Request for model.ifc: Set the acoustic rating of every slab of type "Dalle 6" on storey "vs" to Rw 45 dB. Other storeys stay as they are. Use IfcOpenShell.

First a look at what the model holds.

```python
import ifcopenshell
import ifcopenshell.util.element

model = ifcopenshell.open("model.ifc")
print(model.schema)
storey = next(s for s in model.by_type("IfcBuildingStorey") if s.Name == "vs")
slabs = [e for e in ifcopenshell.util.element.get_decomposition(storey) if e.is_a("IfcSlab")]
seen = {}
for e in slabs:
    element_type = ifcopenshell.util.element.get_type(e)
    key = (element_type.Name if element_type != e and element_type else None, ifcopenshell.util.element.get_pset(e, "Pset_SlabCommon", "AcousticRating"))
    seen[key] = seen.get(key, 0) + 1
for (name, value), count in sorted(seen.items(), key=str):
    print(count, "x", name, "|", value)
```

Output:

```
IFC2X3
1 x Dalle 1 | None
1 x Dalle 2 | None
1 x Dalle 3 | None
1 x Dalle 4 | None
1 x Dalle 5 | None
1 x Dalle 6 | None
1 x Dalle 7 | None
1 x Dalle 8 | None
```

```python
import ifcopenshell
import ifcopenshell.api.pset
import ifcopenshell.util.element

model = ifcopenshell.open("model.ifc")

storey = next(s for s in model.by_type("IfcBuildingStorey") if s.Name == "vs")
slabs = [e for e in ifcopenshell.util.element.get_decomposition(storey) if e.is_a("IfcSlab")]

count = 0
for e in slabs:
    element_type = ifcopenshell.util.element.get_type(e)
    if element_type in (None, e) or element_type.Name != "Dalle 6":
        continue
    # add_pset returns the element's existing set when there is one.
    pset = ifcopenshell.api.pset.add_pset(model, product=e, name="Pset_SlabCommon")
    ifcopenshell.api.pset.edit_pset(model, pset=pset, properties={"AcousticRating": "Rw 45 dB"})
    count += 1

print(count, "slabs updated")

model.write("model_v2.ifc")
```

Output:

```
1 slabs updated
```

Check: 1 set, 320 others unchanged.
